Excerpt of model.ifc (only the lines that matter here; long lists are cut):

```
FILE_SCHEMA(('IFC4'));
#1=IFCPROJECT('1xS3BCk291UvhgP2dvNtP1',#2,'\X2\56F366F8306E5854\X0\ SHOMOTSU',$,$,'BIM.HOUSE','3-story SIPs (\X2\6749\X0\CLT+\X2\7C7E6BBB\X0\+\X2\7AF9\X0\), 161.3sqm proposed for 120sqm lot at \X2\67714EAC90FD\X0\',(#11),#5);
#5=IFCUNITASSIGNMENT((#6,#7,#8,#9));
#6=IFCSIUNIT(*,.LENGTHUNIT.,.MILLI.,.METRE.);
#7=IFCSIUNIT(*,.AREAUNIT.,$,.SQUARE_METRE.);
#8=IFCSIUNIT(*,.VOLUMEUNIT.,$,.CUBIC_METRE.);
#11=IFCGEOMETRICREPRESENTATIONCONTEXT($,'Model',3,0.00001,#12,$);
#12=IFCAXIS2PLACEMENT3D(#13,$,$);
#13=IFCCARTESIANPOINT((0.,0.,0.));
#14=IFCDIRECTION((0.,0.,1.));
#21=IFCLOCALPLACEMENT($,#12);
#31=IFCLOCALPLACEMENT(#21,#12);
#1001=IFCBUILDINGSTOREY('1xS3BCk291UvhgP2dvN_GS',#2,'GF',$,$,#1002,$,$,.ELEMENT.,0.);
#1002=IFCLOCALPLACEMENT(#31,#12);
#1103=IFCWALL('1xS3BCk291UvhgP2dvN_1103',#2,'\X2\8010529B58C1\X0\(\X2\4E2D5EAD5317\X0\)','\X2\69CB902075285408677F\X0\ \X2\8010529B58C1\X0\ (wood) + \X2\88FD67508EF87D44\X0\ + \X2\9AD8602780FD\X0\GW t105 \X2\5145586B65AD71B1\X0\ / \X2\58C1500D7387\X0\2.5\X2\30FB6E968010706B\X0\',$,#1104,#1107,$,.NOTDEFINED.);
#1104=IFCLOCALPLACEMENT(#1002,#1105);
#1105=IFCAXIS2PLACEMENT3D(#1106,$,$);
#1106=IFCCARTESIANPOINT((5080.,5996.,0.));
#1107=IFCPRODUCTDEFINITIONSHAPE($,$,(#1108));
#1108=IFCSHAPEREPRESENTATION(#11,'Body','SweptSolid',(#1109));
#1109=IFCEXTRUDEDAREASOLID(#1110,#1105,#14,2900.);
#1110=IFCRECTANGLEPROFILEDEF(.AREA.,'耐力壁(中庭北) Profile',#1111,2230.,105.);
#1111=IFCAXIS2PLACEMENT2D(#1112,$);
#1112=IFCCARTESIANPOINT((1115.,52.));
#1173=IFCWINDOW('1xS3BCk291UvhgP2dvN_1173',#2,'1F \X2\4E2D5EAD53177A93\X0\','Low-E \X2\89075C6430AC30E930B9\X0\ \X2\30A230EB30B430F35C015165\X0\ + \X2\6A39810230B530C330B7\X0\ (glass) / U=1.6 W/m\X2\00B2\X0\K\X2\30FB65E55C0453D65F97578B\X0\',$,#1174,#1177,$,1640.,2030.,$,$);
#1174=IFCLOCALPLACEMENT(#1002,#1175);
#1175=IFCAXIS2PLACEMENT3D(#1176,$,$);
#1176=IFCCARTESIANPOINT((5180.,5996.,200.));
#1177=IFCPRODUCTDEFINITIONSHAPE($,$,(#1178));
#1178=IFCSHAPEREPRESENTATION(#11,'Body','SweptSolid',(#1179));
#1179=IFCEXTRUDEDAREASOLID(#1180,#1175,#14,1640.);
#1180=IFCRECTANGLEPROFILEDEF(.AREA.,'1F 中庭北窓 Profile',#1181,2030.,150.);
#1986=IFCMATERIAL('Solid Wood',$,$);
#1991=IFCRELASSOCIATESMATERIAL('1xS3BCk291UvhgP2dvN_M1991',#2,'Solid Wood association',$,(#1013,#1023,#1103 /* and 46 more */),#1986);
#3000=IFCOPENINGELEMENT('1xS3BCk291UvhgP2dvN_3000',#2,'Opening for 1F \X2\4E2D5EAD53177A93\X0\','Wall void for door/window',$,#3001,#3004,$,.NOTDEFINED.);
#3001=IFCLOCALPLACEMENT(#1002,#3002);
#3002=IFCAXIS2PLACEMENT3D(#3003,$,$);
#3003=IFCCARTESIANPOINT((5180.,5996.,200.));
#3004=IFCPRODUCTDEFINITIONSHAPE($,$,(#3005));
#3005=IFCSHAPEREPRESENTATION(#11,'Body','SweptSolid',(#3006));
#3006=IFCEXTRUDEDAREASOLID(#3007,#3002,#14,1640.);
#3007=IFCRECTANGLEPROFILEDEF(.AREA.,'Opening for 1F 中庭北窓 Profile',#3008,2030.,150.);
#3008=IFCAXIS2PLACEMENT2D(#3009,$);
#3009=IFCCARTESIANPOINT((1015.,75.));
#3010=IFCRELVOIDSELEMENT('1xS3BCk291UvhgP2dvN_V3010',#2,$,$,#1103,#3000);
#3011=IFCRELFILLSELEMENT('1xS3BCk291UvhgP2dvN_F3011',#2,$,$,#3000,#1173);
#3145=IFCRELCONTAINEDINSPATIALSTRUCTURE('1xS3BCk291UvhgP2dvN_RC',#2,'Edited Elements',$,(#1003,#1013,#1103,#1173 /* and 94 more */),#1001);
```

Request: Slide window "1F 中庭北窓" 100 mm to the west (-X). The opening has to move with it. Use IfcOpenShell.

```python
import ifcopenshell
import ifcopenshell.api.geometry
import ifcopenshell.util.placement
import ifcopenshell.util.unit

model = ifcopenshell.open("model.ifc")
unit_scale = ifcopenshell.util.unit.calculate_unit_scale(model)

window = model.by_guid("1xS3BCk291UvhgP2dvN_1173")
opening = window.FillsVoids[0].RelatingOpeningElement
wall = opening.VoidsElements[0].RelatingBuildingElement

wall_matrix = ifcopenshell.util.placement.get_local_placement(wall.ObjectPlacement)
shift = wall_matrix[:3, 0] * -0.1 / unit_scale
before = ifcopenshell.util.placement.get_local_placement(window.ObjectPlacement)[:3, 3].copy()

# The window is not placed relative to its opening, so move both.
for product in (opening, window):
    matrix = ifcopenshell.util.placement.get_local_placement(product.ObjectPlacement)
    matrix[:3, 3] += shift
    ifcopenshell.api.geometry.edit_object_placement(model, product=product, matrix=matrix, is_si=False)

after = ifcopenshell.util.placement.get_local_placement(window.ObjectPlacement)[:3, 3]
print("window moved by", (after - before).round(3) + 0.0)

model.write("model_rev.ifc")
```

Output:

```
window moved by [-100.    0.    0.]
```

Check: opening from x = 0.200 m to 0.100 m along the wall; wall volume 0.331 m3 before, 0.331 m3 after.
